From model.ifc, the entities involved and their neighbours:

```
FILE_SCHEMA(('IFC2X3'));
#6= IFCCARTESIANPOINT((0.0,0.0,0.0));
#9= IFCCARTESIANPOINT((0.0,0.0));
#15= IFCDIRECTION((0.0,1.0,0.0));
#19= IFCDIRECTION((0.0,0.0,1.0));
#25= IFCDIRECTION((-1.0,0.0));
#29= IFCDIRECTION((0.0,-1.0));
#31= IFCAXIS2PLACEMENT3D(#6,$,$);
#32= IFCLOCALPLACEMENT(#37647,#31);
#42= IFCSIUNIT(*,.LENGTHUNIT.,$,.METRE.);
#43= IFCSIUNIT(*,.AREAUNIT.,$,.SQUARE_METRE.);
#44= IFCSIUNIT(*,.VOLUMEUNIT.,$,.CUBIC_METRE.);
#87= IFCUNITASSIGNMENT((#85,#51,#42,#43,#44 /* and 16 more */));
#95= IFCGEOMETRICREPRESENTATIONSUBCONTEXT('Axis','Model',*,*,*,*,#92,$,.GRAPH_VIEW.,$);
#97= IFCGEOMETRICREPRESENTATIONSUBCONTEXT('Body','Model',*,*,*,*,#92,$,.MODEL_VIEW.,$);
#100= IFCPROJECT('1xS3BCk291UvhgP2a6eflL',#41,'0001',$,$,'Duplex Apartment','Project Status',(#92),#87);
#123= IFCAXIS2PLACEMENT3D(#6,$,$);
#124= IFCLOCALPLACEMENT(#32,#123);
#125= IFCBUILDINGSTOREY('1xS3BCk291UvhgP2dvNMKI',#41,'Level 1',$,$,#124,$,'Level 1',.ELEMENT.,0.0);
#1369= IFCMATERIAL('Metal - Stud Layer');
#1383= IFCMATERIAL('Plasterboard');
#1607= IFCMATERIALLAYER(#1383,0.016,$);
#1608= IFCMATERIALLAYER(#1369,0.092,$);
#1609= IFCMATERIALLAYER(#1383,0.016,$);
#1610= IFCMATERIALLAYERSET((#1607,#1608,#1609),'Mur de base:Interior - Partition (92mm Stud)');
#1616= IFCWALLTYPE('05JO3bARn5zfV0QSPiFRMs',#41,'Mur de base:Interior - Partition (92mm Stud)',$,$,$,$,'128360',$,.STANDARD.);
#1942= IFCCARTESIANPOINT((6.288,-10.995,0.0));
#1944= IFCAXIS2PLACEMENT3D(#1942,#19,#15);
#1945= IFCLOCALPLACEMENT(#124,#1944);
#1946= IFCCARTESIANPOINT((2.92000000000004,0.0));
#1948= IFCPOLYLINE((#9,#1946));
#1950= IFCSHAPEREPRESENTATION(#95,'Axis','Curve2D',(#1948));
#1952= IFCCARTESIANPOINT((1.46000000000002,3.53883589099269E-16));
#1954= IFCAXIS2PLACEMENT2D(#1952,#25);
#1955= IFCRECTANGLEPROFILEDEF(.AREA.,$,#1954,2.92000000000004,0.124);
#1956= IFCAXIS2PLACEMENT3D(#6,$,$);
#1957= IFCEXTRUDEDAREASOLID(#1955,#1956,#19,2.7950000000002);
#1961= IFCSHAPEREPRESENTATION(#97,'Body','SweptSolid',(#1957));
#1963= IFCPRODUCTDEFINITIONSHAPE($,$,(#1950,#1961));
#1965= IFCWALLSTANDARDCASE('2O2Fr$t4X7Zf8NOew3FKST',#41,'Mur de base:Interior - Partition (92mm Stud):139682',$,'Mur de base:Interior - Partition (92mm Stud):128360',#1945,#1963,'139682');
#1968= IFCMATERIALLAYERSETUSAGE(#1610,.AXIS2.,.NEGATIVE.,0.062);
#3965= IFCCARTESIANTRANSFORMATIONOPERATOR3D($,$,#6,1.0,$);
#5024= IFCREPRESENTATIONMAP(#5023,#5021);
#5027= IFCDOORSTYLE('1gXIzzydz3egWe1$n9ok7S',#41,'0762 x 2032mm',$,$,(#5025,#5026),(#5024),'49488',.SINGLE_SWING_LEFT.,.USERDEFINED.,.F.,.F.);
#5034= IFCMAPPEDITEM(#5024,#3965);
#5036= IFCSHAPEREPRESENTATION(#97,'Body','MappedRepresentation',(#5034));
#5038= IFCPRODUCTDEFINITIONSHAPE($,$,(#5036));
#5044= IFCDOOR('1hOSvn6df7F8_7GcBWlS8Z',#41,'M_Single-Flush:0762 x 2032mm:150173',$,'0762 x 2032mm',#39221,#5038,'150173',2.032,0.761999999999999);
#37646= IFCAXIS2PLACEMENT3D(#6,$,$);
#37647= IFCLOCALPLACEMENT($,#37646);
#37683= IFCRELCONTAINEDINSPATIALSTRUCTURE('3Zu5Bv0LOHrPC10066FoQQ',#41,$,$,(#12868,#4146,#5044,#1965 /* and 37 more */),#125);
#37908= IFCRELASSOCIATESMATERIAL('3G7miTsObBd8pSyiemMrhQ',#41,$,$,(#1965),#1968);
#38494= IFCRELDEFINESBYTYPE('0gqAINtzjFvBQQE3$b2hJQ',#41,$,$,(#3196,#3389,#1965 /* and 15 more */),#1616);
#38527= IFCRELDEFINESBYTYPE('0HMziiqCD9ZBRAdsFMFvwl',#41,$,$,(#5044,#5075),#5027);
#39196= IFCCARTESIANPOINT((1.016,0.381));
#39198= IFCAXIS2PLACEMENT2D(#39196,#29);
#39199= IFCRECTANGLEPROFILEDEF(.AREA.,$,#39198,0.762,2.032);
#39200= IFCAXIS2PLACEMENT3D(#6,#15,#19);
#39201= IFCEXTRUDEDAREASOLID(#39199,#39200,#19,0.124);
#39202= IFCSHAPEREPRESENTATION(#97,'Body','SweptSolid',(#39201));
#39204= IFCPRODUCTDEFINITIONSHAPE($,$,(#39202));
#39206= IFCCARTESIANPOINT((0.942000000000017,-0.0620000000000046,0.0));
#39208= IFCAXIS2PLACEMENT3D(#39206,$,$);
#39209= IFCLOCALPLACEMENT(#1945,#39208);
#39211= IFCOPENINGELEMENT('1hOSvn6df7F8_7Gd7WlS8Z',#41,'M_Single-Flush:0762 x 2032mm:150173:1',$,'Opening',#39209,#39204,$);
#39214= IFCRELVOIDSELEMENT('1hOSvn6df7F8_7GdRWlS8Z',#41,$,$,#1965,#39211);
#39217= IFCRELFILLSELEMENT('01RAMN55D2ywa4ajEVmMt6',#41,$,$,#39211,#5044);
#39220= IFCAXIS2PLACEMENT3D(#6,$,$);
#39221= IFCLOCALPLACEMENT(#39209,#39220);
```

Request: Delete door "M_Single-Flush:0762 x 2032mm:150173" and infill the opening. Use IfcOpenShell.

```python
import ifcopenshell
import ifcopenshell.api.feature
import ifcopenshell.api.root
import ifcopenshell.geom
import ifcopenshell.util.shape

model = ifcopenshell.open("model.ifc")
settings = ifcopenshell.geom.settings()


def volume(element):
    """Net volume in cubic metres, openings subtracted."""
    shape = ifcopenshell.geom.create_shape(settings, element)
    return ifcopenshell.util.shape.get_volume(shape.geometry)


door = model.by_id(5044)
opening = door.FillsVoids[0].RelatingOpeningElement
wall = opening.VoidsElements[0].RelatingBuildingElement
before = volume(wall)

ifcopenshell.api.root.remove_product(model, product=door)
ifcopenshell.api.feature.remove_feature(model, feature=opening)

after = volume(wall)

print(f"wall volume {before:.3f} -> {after:.3f} m3")

model.write("model_rev.ifc")
```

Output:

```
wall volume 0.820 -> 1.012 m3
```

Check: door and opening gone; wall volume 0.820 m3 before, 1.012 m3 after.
